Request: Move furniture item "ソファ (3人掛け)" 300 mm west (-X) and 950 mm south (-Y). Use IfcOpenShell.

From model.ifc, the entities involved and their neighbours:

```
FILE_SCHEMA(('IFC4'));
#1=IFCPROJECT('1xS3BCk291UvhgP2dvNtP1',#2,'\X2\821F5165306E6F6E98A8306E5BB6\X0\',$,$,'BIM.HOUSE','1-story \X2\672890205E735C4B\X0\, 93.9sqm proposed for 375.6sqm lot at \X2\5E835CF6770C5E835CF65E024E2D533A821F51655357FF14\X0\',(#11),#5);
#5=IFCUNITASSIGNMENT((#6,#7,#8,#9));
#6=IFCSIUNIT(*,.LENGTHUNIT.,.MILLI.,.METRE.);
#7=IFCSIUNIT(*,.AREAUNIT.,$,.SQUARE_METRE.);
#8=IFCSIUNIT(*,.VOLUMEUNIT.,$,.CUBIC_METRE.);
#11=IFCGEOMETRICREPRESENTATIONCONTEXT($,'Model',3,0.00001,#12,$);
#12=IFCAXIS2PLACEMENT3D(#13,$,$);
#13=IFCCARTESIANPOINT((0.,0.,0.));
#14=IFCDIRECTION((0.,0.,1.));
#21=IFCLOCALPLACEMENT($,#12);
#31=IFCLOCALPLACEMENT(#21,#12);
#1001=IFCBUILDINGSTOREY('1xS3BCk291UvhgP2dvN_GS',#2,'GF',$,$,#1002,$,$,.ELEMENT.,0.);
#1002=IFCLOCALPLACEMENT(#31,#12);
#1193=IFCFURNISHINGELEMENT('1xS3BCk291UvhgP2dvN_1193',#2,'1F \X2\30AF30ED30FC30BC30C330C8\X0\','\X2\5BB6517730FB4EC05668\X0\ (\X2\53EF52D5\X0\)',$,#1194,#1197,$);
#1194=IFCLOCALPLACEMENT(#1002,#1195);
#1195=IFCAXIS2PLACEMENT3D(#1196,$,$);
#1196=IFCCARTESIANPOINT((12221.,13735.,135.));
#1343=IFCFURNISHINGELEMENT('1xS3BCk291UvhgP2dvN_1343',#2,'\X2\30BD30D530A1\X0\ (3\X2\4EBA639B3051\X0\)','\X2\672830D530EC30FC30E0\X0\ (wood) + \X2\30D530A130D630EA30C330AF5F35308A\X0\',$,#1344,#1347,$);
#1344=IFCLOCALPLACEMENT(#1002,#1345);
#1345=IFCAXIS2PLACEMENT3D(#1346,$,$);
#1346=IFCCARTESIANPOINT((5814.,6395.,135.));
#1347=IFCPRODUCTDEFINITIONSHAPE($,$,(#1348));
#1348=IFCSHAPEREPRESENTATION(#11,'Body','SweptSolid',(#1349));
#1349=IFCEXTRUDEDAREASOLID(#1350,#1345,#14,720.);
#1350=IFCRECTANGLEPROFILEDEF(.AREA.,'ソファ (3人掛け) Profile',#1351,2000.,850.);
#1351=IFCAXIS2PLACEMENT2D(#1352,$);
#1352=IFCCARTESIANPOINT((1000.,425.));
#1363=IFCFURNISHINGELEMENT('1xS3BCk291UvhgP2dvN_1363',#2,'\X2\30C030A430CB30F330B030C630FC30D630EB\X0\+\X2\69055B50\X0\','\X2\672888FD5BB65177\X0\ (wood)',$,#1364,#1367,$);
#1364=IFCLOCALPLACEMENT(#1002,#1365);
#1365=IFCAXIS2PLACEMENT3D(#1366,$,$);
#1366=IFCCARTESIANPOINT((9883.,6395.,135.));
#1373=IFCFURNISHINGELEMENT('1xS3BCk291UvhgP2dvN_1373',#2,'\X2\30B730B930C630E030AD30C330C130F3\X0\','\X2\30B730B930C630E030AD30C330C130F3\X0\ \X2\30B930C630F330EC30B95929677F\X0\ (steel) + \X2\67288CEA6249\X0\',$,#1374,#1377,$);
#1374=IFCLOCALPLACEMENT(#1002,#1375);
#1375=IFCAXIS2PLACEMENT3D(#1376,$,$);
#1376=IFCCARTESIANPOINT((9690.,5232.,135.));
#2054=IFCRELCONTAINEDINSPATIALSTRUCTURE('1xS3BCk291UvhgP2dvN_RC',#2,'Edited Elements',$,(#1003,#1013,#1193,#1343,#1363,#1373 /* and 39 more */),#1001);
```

```python
import ifcopenshell
import ifcopenshell.api.geometry
import ifcopenshell.util.placement
import ifcopenshell.util.unit

model = ifcopenshell.open("model.ifc")
unit_scale = ifcopenshell.util.unit.calculate_unit_scale(model)

item = model.by_guid("1xS3BCk291UvhgP2dvN_1343")
matrix = ifcopenshell.util.placement.get_local_placement(item.ObjectPlacement)
matrix[0, 3] -= 0.3 / unit_scale
matrix[1, 3] -= 0.95 / unit_scale
ifcopenshell.api.geometry.edit_object_placement(model, product=item, matrix=matrix, is_si=False)

print(ifcopenshell.util.placement.get_local_placement(item.ObjectPlacement).round(3) + 0.0)

model.write("model_updated.ifc")
```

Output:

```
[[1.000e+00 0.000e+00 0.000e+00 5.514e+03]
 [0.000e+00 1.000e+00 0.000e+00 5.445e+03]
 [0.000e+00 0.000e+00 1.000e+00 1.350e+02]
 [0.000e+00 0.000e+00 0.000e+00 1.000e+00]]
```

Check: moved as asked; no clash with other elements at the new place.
